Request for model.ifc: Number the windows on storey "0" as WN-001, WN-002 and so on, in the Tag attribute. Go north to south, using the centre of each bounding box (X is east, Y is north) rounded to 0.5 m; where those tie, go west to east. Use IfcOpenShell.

First a look at what the model holds.

```python
import ifcopenshell
import ifcopenshell.util.element
import ifcopenshell.util.placement

model = ifcopenshell.open("model.ifc")
print(model.schema)
storey = next(s for s in model.by_type("IfcBuildingStorey") if s.Name == "0")
windows = [e for e in ifcopenshell.util.element.get_decomposition(storey) if e.is_a("IfcWindow")]
for e in sorted(windows, key=lambda e: e.id()):
    origin = ifcopenshell.util.placement.get_local_placement(e.ObjectPlacement)[:3, 3]
    print(e.id(), e.Tag, e.Name, origin.round(2) + 0.0, sep=" | ")
```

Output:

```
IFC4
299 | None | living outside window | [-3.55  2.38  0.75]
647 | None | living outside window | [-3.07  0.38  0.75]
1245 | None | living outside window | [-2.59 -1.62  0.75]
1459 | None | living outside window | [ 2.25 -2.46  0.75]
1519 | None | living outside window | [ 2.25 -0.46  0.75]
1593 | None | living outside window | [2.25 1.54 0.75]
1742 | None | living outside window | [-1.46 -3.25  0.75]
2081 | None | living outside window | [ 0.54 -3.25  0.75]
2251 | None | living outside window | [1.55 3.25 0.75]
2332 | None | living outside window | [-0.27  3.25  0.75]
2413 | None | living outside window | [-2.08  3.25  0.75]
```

```python
import ifcopenshell
import ifcopenshell.geom
import ifcopenshell.util.element
import ifcopenshell.util.shape

model = ifcopenshell.open("model.ifc")
settings = ifcopenshell.geom.settings()
settings.set("use-world-coords", True)


def centre(element):
    shape = ifcopenshell.geom.create_shape(settings, element)
    return ifcopenshell.util.shape.get_bbox_centroid(shape.geometry)


storey = next(s for s in model.by_type("IfcBuildingStorey") if s.Name == "0")
windows = [e for e in ifcopenshell.util.element.get_decomposition(storey) if e.is_a("IfcWindow")]

# Insertion points can sit at a corner or the storey origin, so sort by the geometry (in metres).
centres = {e: centre(e) for e in windows}
windows.sort(key=lambda e: (-round(centres[e][1] / 0.5), centres[e][0]))

for i, e in enumerate(windows, start=1):
    number = f"WN-0{i:02d}"
    e.Tag = number
    print(e.id(), number)

model.write("model-out.ifc")
```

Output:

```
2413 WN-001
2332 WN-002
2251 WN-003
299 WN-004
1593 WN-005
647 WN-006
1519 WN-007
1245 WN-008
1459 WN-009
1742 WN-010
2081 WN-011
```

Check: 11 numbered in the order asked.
